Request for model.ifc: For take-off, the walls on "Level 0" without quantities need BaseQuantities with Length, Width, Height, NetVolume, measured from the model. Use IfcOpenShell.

First a look at what the model holds.

```python
import ifcopenshell
import ifcopenshell.util.element
import ifcopenshell.util.unit

model = ifcopenshell.open("model.ifc")
print(model.schema)
for unit_type in ("LENGTHUNIT", "AREAUNIT", "VOLUMEUNIT"):
    print(unit_type, ifcopenshell.util.unit.calculate_unit_scale(model, unit_type))
storey = next(s for s in model.by_type("IfcBuildingStorey") if s.Name == "Level 0")
walls = [e for e in ifcopenshell.util.element.get_decomposition(storey) if e.is_a("IfcWall")]
for e in sorted(walls, key=lambda e: e.id()):
    print(e.id(), e.is_a(), e.Name, list(ifcopenshell.util.element.get_psets(e, qtos_only=True)), sep=" | ")
```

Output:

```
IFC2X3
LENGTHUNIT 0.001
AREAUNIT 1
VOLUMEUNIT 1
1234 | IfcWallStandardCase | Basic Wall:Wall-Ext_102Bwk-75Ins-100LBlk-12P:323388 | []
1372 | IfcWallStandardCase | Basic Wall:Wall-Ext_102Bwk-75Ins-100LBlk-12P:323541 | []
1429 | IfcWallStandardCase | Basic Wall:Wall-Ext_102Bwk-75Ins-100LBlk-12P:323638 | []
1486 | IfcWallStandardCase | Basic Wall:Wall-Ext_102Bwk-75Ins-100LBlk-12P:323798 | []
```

```python
import ifcopenshell
import ifcopenshell.api.pset
import ifcopenshell.geom
import ifcopenshell.util.element
import ifcopenshell.util.shape
import ifcopenshell.util.unit

model = ifcopenshell.open("model.ifc")
unit_scale = ifcopenshell.util.unit.calculate_unit_scale(model)
volume_scale = ifcopenshell.util.unit.calculate_unit_scale(model, "VOLUMEUNIT")
settings = ifcopenshell.geom.settings()

storey = next(s for s in model.by_type("IfcBuildingStorey") if s.Name == "Level 0")
walls = [e for e in ifcopenshell.util.element.get_decomposition(storey) if e.is_a("IfcWall")]

for e in sorted(walls, key=lambda e: e.id()):
    if ifcopenshell.util.element.get_psets(e, qtos_only=True, should_inherit=False):
        continue
    # Geometry comes back in metres, in the element's own axes.
    shape = ifcopenshell.geom.create_shape(settings, e)
    values = {
        "Length": ifcopenshell.util.shape.get_x(shape.geometry) / unit_scale,
        "Width": ifcopenshell.util.shape.get_y(shape.geometry) / unit_scale,
        "Height": ifcopenshell.util.shape.get_z(shape.geometry) / unit_scale,
        "NetVolume": ifcopenshell.util.shape.get_volume(shape.geometry) / volume_scale,
    }
    qto = ifcopenshell.api.pset.add_qto(model, product=e, name="BaseQuantities")
    ifcopenshell.api.pset.edit_qto(model, qto=qto, properties=values)
    print(e.id(), {k: round(v, 3) for k, v in values.items()})

model.write("model_updated.ifc")
```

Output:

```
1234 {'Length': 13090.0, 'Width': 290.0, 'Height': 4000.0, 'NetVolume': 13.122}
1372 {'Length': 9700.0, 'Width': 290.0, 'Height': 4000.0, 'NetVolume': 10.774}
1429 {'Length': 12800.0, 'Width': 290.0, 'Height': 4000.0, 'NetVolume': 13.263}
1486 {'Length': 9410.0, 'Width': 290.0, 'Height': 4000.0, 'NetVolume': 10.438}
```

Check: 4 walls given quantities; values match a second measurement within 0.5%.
